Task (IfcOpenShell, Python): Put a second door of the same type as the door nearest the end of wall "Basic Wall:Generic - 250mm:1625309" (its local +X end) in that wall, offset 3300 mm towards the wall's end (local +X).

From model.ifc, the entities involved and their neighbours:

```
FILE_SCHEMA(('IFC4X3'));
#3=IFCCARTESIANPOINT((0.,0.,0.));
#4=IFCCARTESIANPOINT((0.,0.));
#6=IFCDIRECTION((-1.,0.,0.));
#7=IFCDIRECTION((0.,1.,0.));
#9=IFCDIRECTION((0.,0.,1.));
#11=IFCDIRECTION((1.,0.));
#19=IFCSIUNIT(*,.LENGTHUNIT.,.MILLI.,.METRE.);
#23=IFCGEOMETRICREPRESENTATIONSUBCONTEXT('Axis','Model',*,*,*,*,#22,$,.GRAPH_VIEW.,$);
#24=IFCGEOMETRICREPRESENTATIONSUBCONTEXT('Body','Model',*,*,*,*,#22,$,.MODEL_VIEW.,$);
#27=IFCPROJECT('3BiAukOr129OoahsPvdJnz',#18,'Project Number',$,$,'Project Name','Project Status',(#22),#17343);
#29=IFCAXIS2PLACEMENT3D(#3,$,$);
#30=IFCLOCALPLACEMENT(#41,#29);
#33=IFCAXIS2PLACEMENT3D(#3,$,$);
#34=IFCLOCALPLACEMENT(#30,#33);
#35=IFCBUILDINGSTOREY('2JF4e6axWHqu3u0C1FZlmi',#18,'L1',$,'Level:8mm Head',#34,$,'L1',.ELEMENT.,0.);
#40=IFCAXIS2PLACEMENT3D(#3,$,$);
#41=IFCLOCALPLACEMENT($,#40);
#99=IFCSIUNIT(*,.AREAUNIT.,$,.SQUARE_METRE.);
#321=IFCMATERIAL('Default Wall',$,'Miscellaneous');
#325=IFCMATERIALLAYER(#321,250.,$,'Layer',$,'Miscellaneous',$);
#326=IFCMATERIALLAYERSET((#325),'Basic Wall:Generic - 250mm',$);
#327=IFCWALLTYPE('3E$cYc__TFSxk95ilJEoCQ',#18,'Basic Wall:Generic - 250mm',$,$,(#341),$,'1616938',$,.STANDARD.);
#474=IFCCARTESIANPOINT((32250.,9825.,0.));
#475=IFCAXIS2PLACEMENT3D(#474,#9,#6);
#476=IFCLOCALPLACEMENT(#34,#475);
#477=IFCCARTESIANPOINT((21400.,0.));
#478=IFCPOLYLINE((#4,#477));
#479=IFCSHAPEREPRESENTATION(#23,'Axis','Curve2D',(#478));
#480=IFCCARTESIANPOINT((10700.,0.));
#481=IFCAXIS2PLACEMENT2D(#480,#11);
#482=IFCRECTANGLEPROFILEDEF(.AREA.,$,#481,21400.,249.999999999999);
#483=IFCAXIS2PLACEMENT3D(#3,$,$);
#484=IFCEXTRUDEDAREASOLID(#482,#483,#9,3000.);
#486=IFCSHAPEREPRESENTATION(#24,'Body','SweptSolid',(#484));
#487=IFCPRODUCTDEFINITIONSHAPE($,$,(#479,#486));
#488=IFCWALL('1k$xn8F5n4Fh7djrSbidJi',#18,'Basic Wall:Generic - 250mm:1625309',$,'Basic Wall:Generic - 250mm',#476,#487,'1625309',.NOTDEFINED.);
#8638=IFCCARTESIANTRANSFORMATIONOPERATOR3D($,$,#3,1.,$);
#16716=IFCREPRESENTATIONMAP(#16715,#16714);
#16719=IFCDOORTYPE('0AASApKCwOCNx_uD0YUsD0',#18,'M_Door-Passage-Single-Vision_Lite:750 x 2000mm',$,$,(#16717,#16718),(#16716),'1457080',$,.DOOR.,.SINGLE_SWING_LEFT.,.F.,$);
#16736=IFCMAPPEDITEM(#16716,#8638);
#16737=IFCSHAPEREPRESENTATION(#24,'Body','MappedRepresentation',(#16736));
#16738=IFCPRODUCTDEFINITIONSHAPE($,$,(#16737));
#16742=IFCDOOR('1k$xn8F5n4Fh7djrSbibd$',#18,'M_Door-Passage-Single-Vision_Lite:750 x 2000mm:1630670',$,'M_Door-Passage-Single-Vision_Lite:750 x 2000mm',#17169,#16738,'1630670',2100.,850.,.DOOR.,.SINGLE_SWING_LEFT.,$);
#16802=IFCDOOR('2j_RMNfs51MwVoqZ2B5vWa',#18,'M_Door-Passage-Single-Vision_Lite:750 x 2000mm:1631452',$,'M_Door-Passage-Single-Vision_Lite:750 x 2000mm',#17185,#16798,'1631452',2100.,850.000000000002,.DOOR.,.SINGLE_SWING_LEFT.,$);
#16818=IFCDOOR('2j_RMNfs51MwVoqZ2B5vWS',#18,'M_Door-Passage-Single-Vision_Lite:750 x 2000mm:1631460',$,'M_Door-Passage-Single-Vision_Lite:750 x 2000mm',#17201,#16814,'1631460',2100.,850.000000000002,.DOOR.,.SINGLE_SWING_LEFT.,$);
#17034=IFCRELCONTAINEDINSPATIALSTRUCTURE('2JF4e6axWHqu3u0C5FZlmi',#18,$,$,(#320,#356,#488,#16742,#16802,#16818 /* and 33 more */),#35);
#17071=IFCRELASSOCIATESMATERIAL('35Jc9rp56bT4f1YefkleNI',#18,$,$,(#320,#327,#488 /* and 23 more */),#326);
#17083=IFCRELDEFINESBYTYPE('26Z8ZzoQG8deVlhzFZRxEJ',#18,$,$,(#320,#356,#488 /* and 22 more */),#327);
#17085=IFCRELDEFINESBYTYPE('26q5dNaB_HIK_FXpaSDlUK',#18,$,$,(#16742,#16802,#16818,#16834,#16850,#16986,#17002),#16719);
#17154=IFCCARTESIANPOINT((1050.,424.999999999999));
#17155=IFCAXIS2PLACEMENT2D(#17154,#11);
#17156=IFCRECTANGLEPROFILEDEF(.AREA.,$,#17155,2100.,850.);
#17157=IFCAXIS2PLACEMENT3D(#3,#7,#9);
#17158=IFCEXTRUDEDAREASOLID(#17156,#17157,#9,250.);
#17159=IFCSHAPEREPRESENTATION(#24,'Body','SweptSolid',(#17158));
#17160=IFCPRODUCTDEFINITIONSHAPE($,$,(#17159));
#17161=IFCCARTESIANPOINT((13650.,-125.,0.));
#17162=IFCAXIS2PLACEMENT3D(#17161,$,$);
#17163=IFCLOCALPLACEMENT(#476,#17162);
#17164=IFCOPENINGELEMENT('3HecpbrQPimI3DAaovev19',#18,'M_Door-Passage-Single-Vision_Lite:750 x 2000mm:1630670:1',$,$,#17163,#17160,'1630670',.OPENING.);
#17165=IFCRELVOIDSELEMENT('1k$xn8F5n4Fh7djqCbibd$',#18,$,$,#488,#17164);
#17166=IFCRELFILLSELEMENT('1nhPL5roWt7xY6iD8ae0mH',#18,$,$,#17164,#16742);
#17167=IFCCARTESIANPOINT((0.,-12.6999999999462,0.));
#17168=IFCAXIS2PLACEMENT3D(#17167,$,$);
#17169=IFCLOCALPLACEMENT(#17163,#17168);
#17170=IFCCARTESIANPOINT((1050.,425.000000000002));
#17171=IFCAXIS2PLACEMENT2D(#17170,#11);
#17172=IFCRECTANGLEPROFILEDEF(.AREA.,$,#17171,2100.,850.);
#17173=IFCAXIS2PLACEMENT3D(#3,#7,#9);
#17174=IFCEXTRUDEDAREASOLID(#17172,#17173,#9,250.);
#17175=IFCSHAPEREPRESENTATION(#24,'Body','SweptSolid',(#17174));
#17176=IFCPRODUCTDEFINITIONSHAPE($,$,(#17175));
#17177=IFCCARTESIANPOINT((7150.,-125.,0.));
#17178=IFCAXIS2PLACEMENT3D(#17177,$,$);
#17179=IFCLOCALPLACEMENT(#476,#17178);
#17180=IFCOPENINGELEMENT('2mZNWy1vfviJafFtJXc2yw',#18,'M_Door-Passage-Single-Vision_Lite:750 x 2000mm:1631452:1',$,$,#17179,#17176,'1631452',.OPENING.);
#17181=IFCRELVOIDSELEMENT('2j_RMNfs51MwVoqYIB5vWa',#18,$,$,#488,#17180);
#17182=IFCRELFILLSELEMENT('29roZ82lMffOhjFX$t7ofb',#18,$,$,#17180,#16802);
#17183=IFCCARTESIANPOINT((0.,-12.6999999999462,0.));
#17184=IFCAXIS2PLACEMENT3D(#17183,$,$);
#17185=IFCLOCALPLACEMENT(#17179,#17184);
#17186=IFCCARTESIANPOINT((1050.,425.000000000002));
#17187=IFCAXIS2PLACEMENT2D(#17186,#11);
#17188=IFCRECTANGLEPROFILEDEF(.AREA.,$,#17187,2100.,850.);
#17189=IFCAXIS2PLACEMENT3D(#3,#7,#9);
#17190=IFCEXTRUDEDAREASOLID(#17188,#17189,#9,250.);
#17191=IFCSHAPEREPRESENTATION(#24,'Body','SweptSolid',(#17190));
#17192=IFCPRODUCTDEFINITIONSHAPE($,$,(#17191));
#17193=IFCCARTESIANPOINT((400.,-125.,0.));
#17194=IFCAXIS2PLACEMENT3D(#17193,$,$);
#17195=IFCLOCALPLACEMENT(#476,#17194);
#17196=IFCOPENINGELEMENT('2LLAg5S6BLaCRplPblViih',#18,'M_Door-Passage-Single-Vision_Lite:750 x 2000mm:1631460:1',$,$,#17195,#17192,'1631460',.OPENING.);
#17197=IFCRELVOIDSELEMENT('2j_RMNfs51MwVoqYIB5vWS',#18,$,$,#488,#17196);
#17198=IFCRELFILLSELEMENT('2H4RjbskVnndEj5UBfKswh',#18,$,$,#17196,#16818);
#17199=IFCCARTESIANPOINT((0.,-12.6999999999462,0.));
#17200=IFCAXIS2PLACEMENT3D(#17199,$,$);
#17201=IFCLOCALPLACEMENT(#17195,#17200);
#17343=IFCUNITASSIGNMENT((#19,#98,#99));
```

```python
import ifcopenshell
import ifcopenshell.api.feature
import ifcopenshell.api.geometry
import ifcopenshell.api.root
import ifcopenshell.geom
import ifcopenshell.util.element
import ifcopenshell.util.placement
import ifcopenshell.util.shape
import ifcopenshell.util.unit

model = ifcopenshell.open("model.ifc")
unit_scale = ifcopenshell.util.unit.calculate_unit_scale(model)
settings = ifcopenshell.geom.settings()


def volume(element):
    """Net volume in cubic metres, openings subtracted."""
    shape = ifcopenshell.geom.create_shape(settings, element)
    return ifcopenshell.util.shape.get_volume(shape.geometry)


def reuse_history(source, copy):
    """copy_class also copies each property set's owner history, people and application; keep the originals."""
    for rel in copy.IsDefinedBy:
        if rel.is_a("IfcRelDefinesByProperties") and (history := rel.RelatingPropertyDefinition.OwnerHistory):
            rel.RelatingPropertyDefinition.OwnerHistory = source.OwnerHistory
            ifcopenshell.util.element.remove_deep2(model, history)


door = model.by_id(16742)
opening = door.FillsVoids[0].RelatingOpeningElement
wall = opening.VoidsElements[0].RelatingBuildingElement
before = volume(wall)
shift = ifcopenshell.util.placement.get_local_placement(wall.ObjectPlacement)[:3, 0] * 3.3 / unit_scale

# copy_class copies the void relationship, type, container and properties, but no geometry.
new_opening = ifcopenshell.api.root.copy_class(model, product=opening)
new_opening.Representation = ifcopenshell.util.element.copy_deep(
    model, opening.Representation, exclude=["IfcGeometricRepresentationContext", "IfcRepresentationMap"]
)
new_opening.Name = "M_Door-Passage-Single-Vision_Lite:750 x 2000mm"
new_opening.Tag = None
new_door = ifcopenshell.api.root.copy_class(model, product=door)
new_door.Representation = ifcopenshell.util.element.copy_deep(
    model, door.Representation, exclude=["IfcGeometricRepresentationContext", "IfcRepresentationMap"]
)
new_door.Name = "M_Door-Passage-Single-Vision_Lite:750 x 2000mm"
new_door.Tag = None
reuse_history(door, new_door)
ifcopenshell.api.feature.add_filling(model, opening=new_opening, element=new_door)

for old, new in ((opening, new_opening), (door, new_door)):
    matrix = ifcopenshell.util.placement.get_local_placement(old.ObjectPlacement)
    matrix[:3, 3] += shift
    ifcopenshell.api.geometry.edit_object_placement(model, product=new, matrix=matrix, is_si=False)

after = volume(wall)

print(f"wall volume {before:.3f} -> {after:.3f} m3")

model.write("model-out.ifc")
```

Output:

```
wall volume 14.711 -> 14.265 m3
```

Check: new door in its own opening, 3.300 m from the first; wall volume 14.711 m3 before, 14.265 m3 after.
